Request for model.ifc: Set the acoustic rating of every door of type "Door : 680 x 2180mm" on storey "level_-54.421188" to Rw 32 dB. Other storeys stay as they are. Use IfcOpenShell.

First a look at what the model holds.

```python
import ifcopenshell
import ifcopenshell.util.element

model = ifcopenshell.open("model.ifc")
print(model.schema)
storey = next(s for s in model.by_type("IfcBuildingStorey") if s.Name == "level_-54.421188")
doors = [e for e in ifcopenshell.util.element.get_decomposition(storey) if e.is_a("IfcDoor")]
seen = {}
for e in doors:
    element_type = ifcopenshell.util.element.get_type(e)
    key = (element_type.Name if element_type != e and element_type else None, ifcopenshell.util.element.get_pset(e, "Pset_DoorCommon", "AcousticRating"))
    seen[key] = seen.get(key, 0) + 1
for (name, value), count in sorted(seen.items(), key=str):
    print(count, "x", name, "|", value)
```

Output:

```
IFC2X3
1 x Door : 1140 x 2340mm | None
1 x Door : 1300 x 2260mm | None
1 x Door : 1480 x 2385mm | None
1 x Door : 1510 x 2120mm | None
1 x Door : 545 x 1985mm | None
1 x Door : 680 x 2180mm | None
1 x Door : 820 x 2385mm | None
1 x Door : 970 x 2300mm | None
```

```python
import ifcopenshell
import ifcopenshell.api.pset
import ifcopenshell.util.element

model = ifcopenshell.open("model.ifc")

storey = next(s for s in model.by_type("IfcBuildingStorey") if s.Name == "level_-54.421188")
doors = [e for e in ifcopenshell.util.element.get_decomposition(storey) if e.is_a("IfcDoor")]

count = 0
for e in doors:
    element_type = ifcopenshell.util.element.get_type(e)
    if element_type in (None, e) or element_type.Name != "Door : 680 x 2180mm":
        continue
    # add_pset returns the element's existing set when there is one.
    pset = ifcopenshell.api.pset.add_pset(model, product=e, name="Pset_DoorCommon")
    ifcopenshell.api.pset.edit_pset(model, pset=pset, properties={"AcousticRating": "Rw 32 dB"})
    count += 1

print(count, "doors updated")

model.write("model_rev.ifc")
```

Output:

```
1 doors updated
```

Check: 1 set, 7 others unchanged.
